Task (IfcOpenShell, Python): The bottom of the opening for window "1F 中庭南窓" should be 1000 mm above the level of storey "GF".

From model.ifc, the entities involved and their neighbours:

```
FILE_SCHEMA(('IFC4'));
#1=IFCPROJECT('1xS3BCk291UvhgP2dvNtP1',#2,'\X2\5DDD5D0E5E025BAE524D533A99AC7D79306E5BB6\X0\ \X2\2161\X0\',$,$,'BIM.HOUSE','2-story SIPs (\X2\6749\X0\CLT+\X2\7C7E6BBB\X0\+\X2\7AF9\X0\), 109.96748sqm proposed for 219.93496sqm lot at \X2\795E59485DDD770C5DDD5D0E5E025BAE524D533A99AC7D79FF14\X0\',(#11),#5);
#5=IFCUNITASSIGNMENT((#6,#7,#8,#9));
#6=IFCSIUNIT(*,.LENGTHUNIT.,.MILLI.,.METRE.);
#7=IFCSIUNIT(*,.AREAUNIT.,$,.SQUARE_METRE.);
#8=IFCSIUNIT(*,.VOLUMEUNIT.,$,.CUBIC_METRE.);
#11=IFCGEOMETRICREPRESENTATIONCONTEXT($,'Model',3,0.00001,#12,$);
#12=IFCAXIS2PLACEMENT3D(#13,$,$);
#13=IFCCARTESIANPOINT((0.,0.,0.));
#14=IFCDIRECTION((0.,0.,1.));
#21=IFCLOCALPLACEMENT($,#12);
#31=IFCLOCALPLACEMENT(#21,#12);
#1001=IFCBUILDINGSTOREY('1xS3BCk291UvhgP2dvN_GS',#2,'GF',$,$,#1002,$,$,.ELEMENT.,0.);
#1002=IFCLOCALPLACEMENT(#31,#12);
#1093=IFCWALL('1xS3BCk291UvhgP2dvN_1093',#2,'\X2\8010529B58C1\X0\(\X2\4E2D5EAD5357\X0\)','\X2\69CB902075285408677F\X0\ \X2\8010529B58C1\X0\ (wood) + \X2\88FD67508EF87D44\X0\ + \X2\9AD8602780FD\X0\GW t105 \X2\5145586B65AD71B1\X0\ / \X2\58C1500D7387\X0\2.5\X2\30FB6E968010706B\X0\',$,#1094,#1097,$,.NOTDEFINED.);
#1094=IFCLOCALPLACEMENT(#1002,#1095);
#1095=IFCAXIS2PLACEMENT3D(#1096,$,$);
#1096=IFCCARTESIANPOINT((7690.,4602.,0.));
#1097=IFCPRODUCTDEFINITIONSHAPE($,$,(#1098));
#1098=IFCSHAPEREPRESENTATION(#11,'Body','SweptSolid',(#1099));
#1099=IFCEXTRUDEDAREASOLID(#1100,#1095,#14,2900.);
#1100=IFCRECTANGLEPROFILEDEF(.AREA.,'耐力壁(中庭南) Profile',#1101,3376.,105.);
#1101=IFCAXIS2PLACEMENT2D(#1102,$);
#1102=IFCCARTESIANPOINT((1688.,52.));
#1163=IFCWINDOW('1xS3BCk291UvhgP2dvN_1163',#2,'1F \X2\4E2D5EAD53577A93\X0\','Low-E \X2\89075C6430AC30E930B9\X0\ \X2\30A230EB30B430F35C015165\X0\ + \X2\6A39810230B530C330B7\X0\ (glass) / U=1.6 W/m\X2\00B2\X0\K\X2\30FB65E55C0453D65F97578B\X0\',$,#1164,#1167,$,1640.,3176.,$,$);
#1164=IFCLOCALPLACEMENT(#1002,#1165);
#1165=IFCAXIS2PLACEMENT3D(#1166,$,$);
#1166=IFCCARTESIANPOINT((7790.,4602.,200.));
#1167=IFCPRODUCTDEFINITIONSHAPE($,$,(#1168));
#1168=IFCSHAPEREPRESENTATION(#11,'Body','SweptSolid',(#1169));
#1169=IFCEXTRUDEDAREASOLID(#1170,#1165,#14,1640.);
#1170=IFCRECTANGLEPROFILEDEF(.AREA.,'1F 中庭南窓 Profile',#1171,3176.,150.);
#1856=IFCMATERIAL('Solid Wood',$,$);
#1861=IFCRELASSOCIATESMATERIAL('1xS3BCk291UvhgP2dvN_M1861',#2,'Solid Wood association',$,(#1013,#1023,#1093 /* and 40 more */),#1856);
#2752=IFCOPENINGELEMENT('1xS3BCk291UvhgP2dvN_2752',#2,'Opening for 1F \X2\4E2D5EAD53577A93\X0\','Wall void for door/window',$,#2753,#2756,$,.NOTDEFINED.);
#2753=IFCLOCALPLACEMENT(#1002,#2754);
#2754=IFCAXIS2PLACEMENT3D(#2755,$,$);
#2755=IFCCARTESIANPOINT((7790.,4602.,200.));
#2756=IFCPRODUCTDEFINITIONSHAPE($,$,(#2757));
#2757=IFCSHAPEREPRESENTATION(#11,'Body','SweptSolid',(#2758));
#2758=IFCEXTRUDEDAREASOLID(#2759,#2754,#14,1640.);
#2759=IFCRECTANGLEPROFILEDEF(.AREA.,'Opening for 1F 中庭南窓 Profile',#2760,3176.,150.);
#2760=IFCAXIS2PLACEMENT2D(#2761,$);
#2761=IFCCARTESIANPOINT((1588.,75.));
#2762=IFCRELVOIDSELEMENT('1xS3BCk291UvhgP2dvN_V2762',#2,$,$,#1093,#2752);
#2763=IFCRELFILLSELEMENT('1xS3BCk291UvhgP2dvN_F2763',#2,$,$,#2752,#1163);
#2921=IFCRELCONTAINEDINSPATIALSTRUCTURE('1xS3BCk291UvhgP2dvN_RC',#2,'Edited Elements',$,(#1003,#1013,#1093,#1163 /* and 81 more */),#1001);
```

```python
import numpy as np
import ifcopenshell
import ifcopenshell.api.geometry
import ifcopenshell.geom
import ifcopenshell.util.element
import ifcopenshell.util.placement
import ifcopenshell.util.shape
import ifcopenshell.util.unit

model = ifcopenshell.open("model.ifc")
unit_scale = ifcopenshell.util.unit.calculate_unit_scale(model)

window = model.by_id(1163)
opening = window.FillsVoids[0].RelatingOpeningElement
storey = ifcopenshell.util.element.get_container(window, ifc_class="IfcBuildingStorey")
level = ifcopenshell.util.placement.get_local_placement(storey.ObjectPlacement)[2, 3]

# The opening's origin need not be at the sill, so measure its lowest point.
shape = ifcopenshell.geom.create_shape(ifcopenshell.geom.settings(), opening)
bottom = ifcopenshell.util.shape.get_shape_bottom_elevation(shape, shape.geometry) / unit_scale
dz = level + 1000.0 - bottom

shift = np.array([0.0, 0.0, dz])
# The window is not placed relative to its opening, so move both.
for product in (opening, window):
    matrix = ifcopenshell.util.placement.get_local_placement(product.ObjectPlacement)
    matrix[:3, 3] += shift
    ifcopenshell.api.geometry.edit_object_placement(model, product=product, matrix=matrix, is_si=False)

print(f"moved by {dz * unit_scale:+.3f} m")

model.write("model_rev.ifc")
```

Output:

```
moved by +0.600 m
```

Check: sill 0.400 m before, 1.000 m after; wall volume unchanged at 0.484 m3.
